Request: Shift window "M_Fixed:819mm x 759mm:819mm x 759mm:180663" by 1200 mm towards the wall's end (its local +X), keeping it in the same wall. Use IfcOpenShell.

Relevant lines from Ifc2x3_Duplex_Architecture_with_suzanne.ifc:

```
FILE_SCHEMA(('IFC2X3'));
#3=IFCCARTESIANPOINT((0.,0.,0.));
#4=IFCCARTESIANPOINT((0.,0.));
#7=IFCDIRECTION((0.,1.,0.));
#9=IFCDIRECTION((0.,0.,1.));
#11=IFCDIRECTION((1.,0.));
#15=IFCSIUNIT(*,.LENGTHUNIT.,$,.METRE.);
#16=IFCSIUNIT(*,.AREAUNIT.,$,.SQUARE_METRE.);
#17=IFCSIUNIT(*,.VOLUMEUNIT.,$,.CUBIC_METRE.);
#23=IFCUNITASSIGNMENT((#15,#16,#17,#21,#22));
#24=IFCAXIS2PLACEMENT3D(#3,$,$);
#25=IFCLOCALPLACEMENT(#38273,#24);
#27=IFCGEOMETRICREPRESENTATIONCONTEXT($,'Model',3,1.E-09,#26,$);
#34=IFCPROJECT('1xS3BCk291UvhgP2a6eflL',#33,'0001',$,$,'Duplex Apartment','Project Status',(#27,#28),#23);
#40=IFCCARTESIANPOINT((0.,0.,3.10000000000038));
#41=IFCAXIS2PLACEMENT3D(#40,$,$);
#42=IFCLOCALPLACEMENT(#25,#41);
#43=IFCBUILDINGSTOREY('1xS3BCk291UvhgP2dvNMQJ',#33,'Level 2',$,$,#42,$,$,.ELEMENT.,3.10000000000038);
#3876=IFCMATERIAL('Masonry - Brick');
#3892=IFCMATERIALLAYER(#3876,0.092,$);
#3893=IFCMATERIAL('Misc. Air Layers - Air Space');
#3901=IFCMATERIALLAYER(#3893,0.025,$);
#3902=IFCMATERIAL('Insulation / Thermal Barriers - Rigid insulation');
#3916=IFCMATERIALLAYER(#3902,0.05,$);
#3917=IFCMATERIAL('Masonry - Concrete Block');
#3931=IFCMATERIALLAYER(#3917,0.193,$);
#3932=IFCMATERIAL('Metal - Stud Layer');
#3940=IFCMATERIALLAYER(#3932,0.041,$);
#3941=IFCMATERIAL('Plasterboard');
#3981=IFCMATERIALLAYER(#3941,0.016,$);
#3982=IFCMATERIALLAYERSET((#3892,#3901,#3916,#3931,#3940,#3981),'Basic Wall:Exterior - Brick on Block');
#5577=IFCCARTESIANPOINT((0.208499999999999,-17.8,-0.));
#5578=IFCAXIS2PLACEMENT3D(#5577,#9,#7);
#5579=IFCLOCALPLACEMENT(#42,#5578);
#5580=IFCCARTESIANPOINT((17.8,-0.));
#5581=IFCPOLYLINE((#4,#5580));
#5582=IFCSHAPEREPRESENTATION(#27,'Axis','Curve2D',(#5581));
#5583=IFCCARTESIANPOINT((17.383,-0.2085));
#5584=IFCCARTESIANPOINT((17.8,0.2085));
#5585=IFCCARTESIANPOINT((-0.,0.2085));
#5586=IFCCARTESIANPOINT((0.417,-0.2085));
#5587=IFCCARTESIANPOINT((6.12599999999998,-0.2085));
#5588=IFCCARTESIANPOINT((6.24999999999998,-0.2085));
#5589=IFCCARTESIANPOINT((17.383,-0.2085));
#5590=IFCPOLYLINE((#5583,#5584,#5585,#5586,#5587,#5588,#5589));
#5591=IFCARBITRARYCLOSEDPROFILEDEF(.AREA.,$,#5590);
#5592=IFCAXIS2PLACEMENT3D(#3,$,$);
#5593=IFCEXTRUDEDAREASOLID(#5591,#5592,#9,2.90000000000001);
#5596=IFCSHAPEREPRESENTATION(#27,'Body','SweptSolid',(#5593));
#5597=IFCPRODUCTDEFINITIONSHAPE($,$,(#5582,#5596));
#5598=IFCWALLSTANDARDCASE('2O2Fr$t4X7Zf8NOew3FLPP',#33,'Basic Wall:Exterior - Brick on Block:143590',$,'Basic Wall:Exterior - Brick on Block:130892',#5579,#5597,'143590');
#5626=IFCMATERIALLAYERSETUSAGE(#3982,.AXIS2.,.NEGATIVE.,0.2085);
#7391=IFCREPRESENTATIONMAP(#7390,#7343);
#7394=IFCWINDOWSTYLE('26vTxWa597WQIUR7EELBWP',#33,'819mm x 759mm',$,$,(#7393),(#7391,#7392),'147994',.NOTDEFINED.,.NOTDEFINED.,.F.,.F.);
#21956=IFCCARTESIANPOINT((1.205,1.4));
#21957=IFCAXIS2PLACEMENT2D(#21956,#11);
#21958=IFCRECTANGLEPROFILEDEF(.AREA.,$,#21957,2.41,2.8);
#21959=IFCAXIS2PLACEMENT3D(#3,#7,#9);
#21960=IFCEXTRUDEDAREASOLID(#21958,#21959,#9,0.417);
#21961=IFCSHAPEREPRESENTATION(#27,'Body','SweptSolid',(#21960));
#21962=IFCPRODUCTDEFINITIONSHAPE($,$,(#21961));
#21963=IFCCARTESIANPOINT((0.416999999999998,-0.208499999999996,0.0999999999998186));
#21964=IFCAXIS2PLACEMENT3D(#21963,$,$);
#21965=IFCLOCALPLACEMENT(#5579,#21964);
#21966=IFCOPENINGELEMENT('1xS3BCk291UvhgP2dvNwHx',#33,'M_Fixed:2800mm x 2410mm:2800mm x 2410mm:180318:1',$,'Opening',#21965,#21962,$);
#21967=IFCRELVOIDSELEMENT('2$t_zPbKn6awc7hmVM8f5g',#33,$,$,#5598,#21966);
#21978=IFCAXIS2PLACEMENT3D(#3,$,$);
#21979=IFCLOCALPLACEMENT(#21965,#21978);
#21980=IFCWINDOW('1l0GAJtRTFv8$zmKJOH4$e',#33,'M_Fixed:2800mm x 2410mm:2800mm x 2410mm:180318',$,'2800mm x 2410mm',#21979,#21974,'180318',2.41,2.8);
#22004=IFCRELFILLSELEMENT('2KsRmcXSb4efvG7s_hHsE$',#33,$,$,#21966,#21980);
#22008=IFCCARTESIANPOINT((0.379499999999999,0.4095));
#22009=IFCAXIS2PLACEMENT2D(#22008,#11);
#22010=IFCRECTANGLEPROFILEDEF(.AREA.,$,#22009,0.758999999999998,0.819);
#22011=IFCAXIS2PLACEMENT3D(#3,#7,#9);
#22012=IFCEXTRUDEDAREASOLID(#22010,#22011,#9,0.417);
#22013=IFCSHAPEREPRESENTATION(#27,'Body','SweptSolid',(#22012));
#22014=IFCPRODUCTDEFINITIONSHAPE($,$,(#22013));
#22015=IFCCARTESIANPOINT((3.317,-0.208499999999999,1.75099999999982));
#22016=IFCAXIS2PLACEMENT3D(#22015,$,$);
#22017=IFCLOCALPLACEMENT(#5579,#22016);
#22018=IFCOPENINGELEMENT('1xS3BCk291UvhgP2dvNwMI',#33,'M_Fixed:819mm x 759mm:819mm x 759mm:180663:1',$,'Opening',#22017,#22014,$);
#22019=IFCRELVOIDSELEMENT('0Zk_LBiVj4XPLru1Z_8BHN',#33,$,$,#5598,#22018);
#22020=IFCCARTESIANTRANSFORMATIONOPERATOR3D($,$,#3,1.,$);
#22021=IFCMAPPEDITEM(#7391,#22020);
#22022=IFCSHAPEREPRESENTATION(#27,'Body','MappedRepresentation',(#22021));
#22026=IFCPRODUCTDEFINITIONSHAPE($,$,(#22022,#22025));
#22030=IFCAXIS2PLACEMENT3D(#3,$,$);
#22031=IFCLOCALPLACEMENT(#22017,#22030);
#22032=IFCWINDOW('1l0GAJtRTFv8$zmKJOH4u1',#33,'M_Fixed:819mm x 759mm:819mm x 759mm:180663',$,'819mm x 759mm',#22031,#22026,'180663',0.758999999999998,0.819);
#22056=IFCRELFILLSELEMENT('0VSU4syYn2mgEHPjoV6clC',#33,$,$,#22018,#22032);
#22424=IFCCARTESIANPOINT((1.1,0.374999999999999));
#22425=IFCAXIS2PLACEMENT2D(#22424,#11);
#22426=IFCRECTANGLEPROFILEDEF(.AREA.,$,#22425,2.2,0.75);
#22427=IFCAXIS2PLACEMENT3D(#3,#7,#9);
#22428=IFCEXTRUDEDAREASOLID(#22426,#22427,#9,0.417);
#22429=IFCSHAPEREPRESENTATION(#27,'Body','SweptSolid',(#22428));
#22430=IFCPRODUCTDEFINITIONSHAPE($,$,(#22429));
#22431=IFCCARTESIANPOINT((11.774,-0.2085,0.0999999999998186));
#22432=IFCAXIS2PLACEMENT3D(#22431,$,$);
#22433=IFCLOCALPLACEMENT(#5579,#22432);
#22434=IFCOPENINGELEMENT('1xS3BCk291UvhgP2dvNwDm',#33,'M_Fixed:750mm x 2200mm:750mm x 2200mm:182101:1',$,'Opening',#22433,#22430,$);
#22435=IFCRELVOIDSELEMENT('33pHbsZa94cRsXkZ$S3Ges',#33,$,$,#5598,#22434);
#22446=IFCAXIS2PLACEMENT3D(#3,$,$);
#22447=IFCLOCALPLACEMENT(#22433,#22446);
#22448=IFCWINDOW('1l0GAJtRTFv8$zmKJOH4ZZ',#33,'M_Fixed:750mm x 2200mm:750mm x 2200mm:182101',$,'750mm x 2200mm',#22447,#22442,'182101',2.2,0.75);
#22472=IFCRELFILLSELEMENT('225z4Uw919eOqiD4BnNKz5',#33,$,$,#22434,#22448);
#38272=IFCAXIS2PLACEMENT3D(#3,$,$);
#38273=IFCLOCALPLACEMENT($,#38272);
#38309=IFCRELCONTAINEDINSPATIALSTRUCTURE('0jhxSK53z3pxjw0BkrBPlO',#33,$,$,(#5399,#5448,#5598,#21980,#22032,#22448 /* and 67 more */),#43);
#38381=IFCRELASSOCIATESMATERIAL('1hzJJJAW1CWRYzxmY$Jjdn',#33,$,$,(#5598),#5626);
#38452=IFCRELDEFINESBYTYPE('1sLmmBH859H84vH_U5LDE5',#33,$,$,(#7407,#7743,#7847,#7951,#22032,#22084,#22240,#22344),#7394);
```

```python
import ifcopenshell
import ifcopenshell.api.geometry
import ifcopenshell.util.placement
import ifcopenshell.util.unit

model = ifcopenshell.open("Ifc2x3_Duplex_Architecture_with_suzanne.ifc")
unit_scale = ifcopenshell.util.unit.calculate_unit_scale(model)

window = model.by_guid("1l0GAJtRTFv8$zmKJOH4u1")
opening = window.FillsVoids[0].RelatingOpeningElement
wall = opening.VoidsElements[0].RelatingBuildingElement

wall_matrix = ifcopenshell.util.placement.get_local_placement(wall.ObjectPlacement)
shift = wall_matrix[:3, 0] * 1.2 / unit_scale
before = ifcopenshell.util.placement.get_local_placement(window.ObjectPlacement)[:3, 3].copy()

# The window is placed relative to its opening, so it follows when the opening moves.
matrix = ifcopenshell.util.placement.get_local_placement(opening.ObjectPlacement)
matrix[:3, 3] += shift
ifcopenshell.api.geometry.edit_object_placement(
    model, product=opening, matrix=matrix, is_si=False, should_transform_children=True
)

after = ifcopenshell.util.placement.get_local_placement(window.ObjectPlacement)[:3, 3]
print("window moved by", (after - before).round(3) + 0.0)

model.write("Ifc2x3_Duplex_Architecture_with_suzanne_rev.ifc")
```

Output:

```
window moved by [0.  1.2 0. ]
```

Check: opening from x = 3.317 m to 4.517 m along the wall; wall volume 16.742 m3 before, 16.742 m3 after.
